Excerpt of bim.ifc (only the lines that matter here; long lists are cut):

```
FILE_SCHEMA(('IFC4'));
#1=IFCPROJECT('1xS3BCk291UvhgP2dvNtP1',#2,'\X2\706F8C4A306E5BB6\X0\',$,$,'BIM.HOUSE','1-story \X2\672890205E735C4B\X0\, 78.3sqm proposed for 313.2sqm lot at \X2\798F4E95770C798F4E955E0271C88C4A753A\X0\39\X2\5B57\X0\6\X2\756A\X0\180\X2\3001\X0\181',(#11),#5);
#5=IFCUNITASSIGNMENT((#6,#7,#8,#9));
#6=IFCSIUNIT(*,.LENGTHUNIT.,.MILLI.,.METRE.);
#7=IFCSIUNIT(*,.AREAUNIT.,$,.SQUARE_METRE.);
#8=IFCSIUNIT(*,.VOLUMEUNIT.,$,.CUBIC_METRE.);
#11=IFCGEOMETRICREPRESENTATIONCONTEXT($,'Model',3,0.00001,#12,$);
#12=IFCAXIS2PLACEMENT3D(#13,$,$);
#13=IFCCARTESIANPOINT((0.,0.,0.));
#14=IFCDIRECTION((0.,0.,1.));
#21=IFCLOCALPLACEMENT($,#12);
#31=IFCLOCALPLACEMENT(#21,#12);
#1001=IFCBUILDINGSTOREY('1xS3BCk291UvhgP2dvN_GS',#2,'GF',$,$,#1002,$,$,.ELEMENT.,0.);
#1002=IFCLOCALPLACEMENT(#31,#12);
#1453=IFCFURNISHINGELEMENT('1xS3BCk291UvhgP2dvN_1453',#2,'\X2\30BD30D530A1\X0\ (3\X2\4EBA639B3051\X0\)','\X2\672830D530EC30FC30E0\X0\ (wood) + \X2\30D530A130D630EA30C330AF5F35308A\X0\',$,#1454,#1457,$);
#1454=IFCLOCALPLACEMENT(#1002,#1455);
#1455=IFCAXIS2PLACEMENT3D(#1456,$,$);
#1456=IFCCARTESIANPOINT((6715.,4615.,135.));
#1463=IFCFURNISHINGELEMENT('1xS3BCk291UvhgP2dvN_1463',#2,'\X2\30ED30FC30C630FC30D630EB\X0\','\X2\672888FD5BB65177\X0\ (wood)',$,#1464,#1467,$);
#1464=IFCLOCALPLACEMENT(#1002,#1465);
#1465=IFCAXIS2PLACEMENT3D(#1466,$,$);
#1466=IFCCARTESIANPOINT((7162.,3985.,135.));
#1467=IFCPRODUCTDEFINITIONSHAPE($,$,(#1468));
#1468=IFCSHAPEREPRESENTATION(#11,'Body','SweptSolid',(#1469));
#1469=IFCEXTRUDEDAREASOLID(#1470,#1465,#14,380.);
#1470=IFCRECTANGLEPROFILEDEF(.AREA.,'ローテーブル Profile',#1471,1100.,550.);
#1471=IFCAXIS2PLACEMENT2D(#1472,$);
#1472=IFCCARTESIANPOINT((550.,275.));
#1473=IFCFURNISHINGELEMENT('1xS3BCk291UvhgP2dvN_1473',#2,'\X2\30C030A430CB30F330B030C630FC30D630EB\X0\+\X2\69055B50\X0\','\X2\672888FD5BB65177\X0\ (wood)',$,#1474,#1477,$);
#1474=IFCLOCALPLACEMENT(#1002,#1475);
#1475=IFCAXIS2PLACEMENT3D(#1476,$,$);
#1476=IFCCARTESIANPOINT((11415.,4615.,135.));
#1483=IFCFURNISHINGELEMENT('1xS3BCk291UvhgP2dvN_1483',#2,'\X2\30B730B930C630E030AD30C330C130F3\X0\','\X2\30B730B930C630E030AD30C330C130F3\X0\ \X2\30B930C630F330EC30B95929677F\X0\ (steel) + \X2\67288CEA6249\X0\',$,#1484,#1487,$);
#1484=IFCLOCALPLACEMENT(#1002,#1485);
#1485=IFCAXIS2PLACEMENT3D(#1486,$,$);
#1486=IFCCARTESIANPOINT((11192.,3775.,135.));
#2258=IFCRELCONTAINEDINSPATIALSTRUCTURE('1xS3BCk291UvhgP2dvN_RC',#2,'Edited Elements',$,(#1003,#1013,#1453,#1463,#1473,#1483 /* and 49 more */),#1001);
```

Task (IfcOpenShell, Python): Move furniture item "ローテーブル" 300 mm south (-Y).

```python
import ifcopenshell
import ifcopenshell.api.geometry
import ifcopenshell.util.placement
import ifcopenshell.util.unit

model = ifcopenshell.open("bim.ifc")
unit_scale = ifcopenshell.util.unit.calculate_unit_scale(model)

item = model.by_guid("1xS3BCk291UvhgP2dvN_1463")
matrix = ifcopenshell.util.placement.get_local_placement(item.ObjectPlacement)
matrix[1, 3] -= 0.3 / unit_scale
ifcopenshell.api.geometry.edit_object_placement(model, product=item, matrix=matrix, is_si=False)

print(ifcopenshell.util.placement.get_local_placement(item.ObjectPlacement).round(3) + 0.0)

model.write("bim_v2.ifc")
```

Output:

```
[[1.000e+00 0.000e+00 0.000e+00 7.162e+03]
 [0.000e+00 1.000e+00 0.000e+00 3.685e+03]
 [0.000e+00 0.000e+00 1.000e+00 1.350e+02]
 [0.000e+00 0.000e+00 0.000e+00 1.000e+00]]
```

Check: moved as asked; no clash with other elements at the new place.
